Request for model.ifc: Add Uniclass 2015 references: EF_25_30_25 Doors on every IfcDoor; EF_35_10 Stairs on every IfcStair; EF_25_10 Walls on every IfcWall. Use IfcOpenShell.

First a look at what the model holds.

```python
import ifcopenshell

model = ifcopenshell.open("model.ifc")
print(model.schema)
print("classifications:", [c.Name for c in model.by_type("IfcClassification")])
for ifc_class in ("IfcDoor", "IfcRoof", "IfcStair", "IfcWall", "IfcWindow"):
    print(ifc_class, len(model.by_type(ifc_class)))
```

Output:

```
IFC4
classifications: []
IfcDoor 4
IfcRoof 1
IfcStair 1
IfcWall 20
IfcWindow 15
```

```python
import ifcopenshell
import ifcopenshell.api.classification

model = ifcopenshell.open("model.ifc")

system = ifcopenshell.api.classification.add_classification(model, classification="Uniclass 2015")

codes = {
    "IfcDoor": ("EF_25_30_25", "Doors"),
    "IfcStair": ("EF_35_10", "Stairs"),
    "IfcWall": ("EF_25_10", "Walls"),
}
for ifc_class, (code, name) in codes.items():
    products = model.by_type(ifc_class)
    ifcopenshell.api.classification.add_reference(
        model, products=products, classification=system, identification=code, name=name
    )
    print(code, len(products))

model.write("model_edited.ifc")
```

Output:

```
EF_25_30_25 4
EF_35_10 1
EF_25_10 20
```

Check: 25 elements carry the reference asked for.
